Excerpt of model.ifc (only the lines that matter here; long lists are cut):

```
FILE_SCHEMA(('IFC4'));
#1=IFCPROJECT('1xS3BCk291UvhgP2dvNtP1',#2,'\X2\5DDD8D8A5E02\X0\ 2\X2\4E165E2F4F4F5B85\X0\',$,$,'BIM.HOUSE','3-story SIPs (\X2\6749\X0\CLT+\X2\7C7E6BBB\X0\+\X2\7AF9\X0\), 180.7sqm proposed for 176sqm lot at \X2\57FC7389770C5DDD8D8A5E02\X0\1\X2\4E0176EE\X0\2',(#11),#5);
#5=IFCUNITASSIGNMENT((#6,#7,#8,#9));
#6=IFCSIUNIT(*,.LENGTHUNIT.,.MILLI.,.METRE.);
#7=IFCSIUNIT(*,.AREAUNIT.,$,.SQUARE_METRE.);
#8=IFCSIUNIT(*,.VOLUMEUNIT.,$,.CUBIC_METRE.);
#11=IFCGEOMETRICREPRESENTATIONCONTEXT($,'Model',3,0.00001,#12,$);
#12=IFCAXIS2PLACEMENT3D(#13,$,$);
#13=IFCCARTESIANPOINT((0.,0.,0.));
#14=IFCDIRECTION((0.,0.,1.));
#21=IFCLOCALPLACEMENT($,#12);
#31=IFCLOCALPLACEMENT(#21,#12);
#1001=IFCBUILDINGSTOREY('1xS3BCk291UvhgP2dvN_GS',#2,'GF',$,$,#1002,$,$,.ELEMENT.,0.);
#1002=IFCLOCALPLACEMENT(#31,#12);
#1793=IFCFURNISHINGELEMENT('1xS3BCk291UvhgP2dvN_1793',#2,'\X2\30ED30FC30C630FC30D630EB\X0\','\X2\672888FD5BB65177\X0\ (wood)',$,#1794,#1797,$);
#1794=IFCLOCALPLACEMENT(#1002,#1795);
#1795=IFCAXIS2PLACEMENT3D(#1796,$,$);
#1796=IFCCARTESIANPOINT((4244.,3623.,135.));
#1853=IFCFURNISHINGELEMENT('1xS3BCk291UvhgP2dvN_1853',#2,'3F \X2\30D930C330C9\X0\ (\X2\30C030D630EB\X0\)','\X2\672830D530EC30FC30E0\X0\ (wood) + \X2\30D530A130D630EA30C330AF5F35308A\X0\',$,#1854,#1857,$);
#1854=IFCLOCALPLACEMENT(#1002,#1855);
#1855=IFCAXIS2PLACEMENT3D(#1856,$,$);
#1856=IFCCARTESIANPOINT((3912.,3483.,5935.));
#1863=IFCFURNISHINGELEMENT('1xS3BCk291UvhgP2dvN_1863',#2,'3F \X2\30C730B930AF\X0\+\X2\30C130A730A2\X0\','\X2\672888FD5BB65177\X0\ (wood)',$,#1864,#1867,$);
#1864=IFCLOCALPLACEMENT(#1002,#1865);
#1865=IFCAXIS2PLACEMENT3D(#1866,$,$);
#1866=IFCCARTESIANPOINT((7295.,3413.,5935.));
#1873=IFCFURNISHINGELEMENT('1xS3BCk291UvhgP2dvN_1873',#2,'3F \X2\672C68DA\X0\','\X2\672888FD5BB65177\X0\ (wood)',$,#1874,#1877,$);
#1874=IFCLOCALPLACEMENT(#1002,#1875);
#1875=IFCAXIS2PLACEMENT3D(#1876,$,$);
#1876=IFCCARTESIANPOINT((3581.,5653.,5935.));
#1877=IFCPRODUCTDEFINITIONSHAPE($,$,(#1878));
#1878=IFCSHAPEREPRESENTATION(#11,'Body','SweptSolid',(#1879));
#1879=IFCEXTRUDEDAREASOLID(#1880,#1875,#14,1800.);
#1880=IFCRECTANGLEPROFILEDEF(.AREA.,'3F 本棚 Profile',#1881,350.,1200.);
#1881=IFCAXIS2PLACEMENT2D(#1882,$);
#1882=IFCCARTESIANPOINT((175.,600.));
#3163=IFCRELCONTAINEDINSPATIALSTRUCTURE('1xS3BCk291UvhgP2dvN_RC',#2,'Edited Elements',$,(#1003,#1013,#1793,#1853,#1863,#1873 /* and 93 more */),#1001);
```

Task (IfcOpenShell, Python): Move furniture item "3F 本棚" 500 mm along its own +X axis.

```python
import ifcopenshell
import ifcopenshell.api.geometry
import ifcopenshell.util.placement

model = ifcopenshell.open("model.ifc")

item = model.by_guid("1xS3BCk291UvhgP2dvN_1873")
matrix = ifcopenshell.util.placement.get_local_placement(item.ObjectPlacement)
matrix[:3, 3] += matrix[:3, 0] * 500.0
ifcopenshell.api.geometry.edit_object_placement(model, product=item, matrix=matrix, is_si=False)

print(ifcopenshell.util.placement.get_local_placement(item.ObjectPlacement).round(3) + 0.0)

model.write("model_edited.ifc")
```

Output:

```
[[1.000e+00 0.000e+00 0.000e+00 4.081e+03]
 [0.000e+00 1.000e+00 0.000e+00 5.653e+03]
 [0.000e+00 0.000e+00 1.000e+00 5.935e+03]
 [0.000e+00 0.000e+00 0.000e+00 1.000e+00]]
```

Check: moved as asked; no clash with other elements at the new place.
